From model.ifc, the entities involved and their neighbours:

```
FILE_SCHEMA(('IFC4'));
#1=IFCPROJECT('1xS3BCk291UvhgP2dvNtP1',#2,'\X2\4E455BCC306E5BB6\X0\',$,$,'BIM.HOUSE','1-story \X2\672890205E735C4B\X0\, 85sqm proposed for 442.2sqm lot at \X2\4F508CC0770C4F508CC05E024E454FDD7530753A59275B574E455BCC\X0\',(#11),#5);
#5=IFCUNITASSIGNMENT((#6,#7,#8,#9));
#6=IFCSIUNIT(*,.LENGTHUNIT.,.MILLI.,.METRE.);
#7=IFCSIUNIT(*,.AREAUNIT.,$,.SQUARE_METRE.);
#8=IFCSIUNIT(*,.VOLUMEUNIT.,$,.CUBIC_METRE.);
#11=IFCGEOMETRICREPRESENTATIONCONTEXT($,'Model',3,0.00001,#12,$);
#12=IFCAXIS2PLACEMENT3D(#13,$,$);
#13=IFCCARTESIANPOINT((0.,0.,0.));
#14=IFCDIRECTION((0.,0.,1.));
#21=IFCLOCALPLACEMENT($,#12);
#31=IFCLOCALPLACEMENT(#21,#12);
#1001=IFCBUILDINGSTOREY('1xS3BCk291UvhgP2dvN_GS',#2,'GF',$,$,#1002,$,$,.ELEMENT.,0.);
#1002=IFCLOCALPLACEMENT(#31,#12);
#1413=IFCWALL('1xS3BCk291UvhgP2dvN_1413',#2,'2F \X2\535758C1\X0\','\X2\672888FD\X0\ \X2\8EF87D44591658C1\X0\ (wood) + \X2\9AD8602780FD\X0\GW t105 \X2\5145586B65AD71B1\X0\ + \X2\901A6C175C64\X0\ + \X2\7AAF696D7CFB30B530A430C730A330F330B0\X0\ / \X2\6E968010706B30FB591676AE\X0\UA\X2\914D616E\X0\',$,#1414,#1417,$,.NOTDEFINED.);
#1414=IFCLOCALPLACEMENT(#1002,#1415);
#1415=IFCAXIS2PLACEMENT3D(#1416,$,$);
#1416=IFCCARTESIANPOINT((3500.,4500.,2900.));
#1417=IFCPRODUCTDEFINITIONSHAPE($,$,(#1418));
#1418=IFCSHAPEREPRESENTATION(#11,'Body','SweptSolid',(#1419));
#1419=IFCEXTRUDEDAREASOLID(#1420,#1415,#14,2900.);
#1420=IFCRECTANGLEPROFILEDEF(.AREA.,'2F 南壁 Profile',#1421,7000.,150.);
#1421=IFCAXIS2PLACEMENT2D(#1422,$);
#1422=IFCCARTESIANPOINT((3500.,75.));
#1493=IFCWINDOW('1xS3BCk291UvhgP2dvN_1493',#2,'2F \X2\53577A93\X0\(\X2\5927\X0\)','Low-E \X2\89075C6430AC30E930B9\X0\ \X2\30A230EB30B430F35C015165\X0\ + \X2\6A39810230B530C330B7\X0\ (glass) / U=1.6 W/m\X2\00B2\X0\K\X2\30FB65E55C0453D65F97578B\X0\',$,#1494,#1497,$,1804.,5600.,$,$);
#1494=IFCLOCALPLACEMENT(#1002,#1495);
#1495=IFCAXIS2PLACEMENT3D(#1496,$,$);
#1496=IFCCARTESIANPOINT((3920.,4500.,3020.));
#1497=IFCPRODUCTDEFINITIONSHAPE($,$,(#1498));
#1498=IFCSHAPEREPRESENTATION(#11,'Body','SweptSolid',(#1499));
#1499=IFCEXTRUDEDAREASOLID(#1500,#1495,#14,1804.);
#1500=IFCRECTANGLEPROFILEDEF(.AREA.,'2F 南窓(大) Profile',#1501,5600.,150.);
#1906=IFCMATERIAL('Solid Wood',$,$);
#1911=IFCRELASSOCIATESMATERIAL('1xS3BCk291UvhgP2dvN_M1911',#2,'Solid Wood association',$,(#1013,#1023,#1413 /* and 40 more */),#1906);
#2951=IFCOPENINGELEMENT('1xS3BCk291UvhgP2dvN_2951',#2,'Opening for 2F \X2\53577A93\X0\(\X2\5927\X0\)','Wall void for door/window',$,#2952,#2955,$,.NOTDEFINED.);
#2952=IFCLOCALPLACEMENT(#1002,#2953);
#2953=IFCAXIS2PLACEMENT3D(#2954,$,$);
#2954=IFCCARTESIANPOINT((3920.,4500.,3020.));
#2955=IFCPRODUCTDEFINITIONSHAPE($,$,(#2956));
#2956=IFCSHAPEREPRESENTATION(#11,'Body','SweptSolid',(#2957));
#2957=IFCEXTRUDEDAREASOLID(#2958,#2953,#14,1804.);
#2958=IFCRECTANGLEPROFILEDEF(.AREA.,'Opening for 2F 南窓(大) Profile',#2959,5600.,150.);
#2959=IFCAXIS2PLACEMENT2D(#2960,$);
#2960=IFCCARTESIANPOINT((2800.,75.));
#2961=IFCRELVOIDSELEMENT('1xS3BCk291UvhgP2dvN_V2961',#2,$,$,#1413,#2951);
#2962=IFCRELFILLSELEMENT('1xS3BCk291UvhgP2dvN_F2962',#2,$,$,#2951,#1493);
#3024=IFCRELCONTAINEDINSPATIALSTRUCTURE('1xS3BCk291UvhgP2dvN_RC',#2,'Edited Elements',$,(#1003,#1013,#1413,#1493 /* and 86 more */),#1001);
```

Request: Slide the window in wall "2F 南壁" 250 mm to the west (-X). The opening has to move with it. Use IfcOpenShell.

```python
import ifcopenshell
import ifcopenshell.api.geometry
import ifcopenshell.util.placement
import ifcopenshell.util.unit

model = ifcopenshell.open("model.ifc")
unit_scale = ifcopenshell.util.unit.calculate_unit_scale(model)

window = model.by_guid("1xS3BCk291UvhgP2dvN_1493")
opening = window.FillsVoids[0].RelatingOpeningElement
wall = opening.VoidsElements[0].RelatingBuildingElement

wall_matrix = ifcopenshell.util.placement.get_local_placement(wall.ObjectPlacement)
shift = wall_matrix[:3, 0] * -0.25 / unit_scale
before = ifcopenshell.util.placement.get_local_placement(window.ObjectPlacement)[:3, 3].copy()

# The window is not placed relative to its opening, so move both.
for product in (opening, window):
    matrix = ifcopenshell.util.placement.get_local_placement(product.ObjectPlacement)
    matrix[:3, 3] += shift
    ifcopenshell.api.geometry.edit_object_placement(model, product=product, matrix=matrix, is_si=False)

after = ifcopenshell.util.placement.get_local_placement(window.ObjectPlacement)[:3, 3]
print("window moved by", (after - before).round(3) + 0.0)

model.write("model-out.ifc")
```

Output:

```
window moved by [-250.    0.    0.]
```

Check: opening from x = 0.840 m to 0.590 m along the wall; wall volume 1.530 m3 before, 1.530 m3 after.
